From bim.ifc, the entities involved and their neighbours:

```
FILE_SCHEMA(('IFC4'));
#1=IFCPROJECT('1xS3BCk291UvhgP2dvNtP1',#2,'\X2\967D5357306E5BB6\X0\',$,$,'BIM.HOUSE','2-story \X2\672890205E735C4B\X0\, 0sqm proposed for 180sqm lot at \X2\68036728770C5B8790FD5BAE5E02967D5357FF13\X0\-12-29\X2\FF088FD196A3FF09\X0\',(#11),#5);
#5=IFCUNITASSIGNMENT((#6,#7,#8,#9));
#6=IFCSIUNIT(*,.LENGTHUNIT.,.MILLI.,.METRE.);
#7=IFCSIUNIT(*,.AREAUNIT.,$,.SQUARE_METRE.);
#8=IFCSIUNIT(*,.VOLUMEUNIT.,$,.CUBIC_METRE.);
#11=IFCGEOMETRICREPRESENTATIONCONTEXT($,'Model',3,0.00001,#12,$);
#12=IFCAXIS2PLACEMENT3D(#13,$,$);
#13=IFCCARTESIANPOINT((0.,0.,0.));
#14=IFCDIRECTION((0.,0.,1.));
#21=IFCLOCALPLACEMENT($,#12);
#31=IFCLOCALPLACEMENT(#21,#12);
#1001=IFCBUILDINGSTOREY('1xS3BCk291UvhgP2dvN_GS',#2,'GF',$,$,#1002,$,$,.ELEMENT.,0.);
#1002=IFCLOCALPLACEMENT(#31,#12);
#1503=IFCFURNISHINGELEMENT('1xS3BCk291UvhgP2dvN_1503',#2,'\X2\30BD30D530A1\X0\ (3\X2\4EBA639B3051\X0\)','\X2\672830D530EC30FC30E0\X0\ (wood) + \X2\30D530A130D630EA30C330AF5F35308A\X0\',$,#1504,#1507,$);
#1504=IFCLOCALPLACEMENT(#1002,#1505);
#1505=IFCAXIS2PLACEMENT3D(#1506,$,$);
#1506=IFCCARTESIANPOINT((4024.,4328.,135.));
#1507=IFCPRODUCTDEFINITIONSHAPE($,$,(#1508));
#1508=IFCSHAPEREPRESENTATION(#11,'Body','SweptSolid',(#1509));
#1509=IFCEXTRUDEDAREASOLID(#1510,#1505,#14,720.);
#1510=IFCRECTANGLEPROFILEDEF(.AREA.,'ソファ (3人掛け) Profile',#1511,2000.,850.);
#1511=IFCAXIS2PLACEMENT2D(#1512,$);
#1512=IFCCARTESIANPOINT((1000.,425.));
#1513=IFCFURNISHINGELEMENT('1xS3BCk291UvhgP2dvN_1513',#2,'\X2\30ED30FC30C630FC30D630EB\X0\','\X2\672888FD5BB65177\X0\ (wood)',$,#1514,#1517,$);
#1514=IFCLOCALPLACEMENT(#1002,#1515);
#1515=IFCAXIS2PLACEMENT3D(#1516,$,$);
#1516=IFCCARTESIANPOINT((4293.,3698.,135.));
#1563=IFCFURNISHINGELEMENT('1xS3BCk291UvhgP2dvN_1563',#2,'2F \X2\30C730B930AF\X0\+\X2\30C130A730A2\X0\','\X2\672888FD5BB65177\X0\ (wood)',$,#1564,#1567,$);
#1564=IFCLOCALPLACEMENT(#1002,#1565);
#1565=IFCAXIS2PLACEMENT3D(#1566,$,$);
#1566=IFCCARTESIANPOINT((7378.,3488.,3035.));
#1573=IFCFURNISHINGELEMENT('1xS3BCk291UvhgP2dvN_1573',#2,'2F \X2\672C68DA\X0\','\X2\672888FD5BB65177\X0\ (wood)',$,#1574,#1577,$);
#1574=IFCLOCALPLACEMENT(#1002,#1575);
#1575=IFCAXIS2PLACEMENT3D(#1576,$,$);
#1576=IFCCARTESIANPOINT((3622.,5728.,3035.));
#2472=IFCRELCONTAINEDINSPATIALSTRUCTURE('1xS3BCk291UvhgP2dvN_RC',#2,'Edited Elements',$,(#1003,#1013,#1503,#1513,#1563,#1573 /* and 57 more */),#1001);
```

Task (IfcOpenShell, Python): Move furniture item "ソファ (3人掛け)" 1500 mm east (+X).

```python
import ifcopenshell
import ifcopenshell.api.geometry
import ifcopenshell.util.placement
import ifcopenshell.util.unit

model = ifcopenshell.open("bim.ifc")
unit_scale = ifcopenshell.util.unit.calculate_unit_scale(model)

item = model.by_guid("1xS3BCk291UvhgP2dvN_1503")
matrix = ifcopenshell.util.placement.get_local_placement(item.ObjectPlacement)
matrix[0, 3] += 1.5 / unit_scale
ifcopenshell.api.geometry.edit_object_placement(model, product=item, matrix=matrix, is_si=False)

print(ifcopenshell.util.placement.get_local_placement(item.ObjectPlacement).round(3) + 0.0)

model.write("bim-out.ifc")
```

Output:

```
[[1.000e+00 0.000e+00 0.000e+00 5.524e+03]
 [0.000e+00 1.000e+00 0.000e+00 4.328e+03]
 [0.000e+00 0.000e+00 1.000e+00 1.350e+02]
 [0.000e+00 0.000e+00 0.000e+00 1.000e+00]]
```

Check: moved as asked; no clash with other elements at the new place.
